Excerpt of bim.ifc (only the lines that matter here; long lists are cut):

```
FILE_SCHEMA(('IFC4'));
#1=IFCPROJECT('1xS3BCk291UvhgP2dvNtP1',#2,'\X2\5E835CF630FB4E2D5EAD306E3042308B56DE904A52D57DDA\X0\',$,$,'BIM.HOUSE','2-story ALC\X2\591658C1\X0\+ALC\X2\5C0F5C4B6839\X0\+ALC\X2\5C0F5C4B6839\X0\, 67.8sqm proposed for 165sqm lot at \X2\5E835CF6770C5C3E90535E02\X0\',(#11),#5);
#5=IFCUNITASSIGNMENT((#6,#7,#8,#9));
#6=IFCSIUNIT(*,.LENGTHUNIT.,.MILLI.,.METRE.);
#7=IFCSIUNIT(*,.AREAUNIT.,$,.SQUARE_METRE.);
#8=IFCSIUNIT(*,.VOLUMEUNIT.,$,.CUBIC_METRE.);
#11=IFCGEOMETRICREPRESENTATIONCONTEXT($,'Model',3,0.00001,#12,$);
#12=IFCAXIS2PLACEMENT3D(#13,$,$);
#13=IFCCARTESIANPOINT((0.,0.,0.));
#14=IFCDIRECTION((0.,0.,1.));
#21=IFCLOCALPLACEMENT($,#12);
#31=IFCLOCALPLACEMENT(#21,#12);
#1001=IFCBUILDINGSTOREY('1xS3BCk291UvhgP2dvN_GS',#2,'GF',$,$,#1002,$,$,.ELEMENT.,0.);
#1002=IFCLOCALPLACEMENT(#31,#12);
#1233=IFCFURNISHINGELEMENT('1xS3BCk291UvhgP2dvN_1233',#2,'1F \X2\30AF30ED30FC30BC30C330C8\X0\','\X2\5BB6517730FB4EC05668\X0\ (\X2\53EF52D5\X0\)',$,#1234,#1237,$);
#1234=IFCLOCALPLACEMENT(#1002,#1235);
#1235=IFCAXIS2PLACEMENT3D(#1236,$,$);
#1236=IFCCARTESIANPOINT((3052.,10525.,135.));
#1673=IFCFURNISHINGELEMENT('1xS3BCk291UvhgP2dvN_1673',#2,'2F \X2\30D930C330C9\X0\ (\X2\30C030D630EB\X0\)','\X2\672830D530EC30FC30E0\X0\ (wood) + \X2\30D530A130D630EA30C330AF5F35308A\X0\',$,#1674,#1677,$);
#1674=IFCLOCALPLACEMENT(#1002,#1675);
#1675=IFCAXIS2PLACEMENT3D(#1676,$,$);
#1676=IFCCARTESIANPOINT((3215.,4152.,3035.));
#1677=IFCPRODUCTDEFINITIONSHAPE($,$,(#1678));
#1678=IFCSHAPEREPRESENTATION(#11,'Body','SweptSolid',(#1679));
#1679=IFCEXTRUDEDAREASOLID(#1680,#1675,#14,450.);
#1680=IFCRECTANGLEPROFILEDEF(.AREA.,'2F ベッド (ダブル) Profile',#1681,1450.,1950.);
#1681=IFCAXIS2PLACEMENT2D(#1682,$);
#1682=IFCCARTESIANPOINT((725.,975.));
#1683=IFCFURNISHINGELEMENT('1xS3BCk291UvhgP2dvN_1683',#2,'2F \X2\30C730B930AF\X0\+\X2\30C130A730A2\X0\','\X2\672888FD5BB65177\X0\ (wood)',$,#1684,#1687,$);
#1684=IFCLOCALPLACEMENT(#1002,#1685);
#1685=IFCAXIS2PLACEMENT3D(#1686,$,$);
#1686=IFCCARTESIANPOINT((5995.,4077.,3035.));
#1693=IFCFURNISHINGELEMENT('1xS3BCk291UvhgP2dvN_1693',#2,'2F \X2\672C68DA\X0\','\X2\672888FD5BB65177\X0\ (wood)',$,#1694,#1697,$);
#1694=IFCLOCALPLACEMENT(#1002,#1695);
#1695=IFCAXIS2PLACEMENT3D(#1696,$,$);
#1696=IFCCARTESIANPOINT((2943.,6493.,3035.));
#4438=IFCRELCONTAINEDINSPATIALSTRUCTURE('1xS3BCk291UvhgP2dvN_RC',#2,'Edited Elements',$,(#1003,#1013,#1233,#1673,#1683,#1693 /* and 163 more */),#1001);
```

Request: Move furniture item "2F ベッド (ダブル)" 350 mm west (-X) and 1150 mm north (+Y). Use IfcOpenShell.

```python
import ifcopenshell
import ifcopenshell.api.geometry
import ifcopenshell.util.placement
import ifcopenshell.util.unit

model = ifcopenshell.open("bim.ifc")
unit_scale = ifcopenshell.util.unit.calculate_unit_scale(model)

item = model.by_id(1673)
matrix = ifcopenshell.util.placement.get_local_placement(item.ObjectPlacement)
matrix[0, 3] -= 0.35 / unit_scale
matrix[1, 3] += 1.15 / unit_scale
ifcopenshell.api.geometry.edit_object_placement(model, product=item, matrix=matrix, is_si=False)

print(ifcopenshell.util.placement.get_local_placement(item.ObjectPlacement).round(3) + 0.0)

model.write("bim_updated.ifc")
```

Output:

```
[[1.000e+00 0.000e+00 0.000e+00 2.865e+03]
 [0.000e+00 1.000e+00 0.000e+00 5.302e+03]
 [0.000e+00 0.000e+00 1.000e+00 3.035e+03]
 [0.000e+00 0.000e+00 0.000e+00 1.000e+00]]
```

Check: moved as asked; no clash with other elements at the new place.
